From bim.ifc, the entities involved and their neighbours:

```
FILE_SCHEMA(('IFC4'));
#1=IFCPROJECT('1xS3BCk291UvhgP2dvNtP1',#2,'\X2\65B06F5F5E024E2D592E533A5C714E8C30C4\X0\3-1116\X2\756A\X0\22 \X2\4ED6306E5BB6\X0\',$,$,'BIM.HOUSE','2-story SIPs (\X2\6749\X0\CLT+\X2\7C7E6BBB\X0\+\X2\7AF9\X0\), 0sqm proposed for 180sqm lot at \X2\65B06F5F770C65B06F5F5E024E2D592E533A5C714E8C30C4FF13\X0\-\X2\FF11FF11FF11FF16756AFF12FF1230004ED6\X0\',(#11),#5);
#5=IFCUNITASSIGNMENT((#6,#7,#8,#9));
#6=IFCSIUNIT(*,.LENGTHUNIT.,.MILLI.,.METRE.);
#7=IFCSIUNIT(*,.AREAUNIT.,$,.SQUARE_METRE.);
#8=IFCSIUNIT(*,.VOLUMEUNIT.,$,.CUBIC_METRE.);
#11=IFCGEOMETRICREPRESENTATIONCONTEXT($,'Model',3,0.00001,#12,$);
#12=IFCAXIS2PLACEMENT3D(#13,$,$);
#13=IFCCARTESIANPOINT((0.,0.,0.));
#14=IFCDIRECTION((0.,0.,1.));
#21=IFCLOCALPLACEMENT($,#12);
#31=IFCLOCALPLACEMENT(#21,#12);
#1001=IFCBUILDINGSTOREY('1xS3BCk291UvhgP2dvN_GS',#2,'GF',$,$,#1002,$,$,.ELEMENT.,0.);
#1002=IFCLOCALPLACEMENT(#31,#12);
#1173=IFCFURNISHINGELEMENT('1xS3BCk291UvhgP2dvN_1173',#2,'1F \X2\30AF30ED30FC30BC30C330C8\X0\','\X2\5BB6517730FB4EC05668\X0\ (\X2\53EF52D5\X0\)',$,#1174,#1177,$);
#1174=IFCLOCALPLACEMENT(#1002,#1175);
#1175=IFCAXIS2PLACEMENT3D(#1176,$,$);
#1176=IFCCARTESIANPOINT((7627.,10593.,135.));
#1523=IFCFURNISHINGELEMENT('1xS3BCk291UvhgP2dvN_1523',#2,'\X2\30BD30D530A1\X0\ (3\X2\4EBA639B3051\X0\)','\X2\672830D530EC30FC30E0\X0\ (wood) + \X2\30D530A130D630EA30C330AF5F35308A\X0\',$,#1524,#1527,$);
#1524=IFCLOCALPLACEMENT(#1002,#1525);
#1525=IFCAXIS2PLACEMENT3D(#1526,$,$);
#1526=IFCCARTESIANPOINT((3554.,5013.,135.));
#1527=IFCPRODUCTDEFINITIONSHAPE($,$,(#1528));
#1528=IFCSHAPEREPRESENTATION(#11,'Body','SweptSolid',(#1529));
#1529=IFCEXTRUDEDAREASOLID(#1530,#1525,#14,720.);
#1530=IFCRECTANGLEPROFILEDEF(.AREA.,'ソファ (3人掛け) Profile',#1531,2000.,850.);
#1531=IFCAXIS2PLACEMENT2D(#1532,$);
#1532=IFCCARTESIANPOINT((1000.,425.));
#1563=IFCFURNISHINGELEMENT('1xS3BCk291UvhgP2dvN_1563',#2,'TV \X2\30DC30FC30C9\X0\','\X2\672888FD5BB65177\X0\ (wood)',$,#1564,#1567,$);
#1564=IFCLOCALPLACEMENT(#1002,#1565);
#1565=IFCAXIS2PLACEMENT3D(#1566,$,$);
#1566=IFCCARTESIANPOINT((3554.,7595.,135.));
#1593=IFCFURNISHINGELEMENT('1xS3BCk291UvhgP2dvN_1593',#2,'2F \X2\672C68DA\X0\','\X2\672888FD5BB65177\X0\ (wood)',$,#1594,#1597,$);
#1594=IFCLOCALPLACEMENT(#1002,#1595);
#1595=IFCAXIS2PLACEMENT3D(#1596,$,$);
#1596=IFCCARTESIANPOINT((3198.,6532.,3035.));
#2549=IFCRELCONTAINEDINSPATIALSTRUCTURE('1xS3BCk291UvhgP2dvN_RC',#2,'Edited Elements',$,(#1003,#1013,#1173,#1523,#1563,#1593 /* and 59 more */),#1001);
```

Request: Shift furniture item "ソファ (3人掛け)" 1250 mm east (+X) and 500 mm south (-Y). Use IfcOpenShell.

```python
import ifcopenshell
import ifcopenshell.api.geometry
import ifcopenshell.util.placement

model = ifcopenshell.open("bim.ifc")

item = model.by_guid("1xS3BCk291UvhgP2dvN_1523")
matrix = ifcopenshell.util.placement.get_local_placement(item.ObjectPlacement)
matrix[0, 3] += 1250.0
matrix[1, 3] -= 500.0
ifcopenshell.api.geometry.edit_object_placement(model, product=item, matrix=matrix, is_si=False)

print(ifcopenshell.util.placement.get_local_placement(item.ObjectPlacement).round(3) + 0.0)

model.write("bim_v2.ifc")
```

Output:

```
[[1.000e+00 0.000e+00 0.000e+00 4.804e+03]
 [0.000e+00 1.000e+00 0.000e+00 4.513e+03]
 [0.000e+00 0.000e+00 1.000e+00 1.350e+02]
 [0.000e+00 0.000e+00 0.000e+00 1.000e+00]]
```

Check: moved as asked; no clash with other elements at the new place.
